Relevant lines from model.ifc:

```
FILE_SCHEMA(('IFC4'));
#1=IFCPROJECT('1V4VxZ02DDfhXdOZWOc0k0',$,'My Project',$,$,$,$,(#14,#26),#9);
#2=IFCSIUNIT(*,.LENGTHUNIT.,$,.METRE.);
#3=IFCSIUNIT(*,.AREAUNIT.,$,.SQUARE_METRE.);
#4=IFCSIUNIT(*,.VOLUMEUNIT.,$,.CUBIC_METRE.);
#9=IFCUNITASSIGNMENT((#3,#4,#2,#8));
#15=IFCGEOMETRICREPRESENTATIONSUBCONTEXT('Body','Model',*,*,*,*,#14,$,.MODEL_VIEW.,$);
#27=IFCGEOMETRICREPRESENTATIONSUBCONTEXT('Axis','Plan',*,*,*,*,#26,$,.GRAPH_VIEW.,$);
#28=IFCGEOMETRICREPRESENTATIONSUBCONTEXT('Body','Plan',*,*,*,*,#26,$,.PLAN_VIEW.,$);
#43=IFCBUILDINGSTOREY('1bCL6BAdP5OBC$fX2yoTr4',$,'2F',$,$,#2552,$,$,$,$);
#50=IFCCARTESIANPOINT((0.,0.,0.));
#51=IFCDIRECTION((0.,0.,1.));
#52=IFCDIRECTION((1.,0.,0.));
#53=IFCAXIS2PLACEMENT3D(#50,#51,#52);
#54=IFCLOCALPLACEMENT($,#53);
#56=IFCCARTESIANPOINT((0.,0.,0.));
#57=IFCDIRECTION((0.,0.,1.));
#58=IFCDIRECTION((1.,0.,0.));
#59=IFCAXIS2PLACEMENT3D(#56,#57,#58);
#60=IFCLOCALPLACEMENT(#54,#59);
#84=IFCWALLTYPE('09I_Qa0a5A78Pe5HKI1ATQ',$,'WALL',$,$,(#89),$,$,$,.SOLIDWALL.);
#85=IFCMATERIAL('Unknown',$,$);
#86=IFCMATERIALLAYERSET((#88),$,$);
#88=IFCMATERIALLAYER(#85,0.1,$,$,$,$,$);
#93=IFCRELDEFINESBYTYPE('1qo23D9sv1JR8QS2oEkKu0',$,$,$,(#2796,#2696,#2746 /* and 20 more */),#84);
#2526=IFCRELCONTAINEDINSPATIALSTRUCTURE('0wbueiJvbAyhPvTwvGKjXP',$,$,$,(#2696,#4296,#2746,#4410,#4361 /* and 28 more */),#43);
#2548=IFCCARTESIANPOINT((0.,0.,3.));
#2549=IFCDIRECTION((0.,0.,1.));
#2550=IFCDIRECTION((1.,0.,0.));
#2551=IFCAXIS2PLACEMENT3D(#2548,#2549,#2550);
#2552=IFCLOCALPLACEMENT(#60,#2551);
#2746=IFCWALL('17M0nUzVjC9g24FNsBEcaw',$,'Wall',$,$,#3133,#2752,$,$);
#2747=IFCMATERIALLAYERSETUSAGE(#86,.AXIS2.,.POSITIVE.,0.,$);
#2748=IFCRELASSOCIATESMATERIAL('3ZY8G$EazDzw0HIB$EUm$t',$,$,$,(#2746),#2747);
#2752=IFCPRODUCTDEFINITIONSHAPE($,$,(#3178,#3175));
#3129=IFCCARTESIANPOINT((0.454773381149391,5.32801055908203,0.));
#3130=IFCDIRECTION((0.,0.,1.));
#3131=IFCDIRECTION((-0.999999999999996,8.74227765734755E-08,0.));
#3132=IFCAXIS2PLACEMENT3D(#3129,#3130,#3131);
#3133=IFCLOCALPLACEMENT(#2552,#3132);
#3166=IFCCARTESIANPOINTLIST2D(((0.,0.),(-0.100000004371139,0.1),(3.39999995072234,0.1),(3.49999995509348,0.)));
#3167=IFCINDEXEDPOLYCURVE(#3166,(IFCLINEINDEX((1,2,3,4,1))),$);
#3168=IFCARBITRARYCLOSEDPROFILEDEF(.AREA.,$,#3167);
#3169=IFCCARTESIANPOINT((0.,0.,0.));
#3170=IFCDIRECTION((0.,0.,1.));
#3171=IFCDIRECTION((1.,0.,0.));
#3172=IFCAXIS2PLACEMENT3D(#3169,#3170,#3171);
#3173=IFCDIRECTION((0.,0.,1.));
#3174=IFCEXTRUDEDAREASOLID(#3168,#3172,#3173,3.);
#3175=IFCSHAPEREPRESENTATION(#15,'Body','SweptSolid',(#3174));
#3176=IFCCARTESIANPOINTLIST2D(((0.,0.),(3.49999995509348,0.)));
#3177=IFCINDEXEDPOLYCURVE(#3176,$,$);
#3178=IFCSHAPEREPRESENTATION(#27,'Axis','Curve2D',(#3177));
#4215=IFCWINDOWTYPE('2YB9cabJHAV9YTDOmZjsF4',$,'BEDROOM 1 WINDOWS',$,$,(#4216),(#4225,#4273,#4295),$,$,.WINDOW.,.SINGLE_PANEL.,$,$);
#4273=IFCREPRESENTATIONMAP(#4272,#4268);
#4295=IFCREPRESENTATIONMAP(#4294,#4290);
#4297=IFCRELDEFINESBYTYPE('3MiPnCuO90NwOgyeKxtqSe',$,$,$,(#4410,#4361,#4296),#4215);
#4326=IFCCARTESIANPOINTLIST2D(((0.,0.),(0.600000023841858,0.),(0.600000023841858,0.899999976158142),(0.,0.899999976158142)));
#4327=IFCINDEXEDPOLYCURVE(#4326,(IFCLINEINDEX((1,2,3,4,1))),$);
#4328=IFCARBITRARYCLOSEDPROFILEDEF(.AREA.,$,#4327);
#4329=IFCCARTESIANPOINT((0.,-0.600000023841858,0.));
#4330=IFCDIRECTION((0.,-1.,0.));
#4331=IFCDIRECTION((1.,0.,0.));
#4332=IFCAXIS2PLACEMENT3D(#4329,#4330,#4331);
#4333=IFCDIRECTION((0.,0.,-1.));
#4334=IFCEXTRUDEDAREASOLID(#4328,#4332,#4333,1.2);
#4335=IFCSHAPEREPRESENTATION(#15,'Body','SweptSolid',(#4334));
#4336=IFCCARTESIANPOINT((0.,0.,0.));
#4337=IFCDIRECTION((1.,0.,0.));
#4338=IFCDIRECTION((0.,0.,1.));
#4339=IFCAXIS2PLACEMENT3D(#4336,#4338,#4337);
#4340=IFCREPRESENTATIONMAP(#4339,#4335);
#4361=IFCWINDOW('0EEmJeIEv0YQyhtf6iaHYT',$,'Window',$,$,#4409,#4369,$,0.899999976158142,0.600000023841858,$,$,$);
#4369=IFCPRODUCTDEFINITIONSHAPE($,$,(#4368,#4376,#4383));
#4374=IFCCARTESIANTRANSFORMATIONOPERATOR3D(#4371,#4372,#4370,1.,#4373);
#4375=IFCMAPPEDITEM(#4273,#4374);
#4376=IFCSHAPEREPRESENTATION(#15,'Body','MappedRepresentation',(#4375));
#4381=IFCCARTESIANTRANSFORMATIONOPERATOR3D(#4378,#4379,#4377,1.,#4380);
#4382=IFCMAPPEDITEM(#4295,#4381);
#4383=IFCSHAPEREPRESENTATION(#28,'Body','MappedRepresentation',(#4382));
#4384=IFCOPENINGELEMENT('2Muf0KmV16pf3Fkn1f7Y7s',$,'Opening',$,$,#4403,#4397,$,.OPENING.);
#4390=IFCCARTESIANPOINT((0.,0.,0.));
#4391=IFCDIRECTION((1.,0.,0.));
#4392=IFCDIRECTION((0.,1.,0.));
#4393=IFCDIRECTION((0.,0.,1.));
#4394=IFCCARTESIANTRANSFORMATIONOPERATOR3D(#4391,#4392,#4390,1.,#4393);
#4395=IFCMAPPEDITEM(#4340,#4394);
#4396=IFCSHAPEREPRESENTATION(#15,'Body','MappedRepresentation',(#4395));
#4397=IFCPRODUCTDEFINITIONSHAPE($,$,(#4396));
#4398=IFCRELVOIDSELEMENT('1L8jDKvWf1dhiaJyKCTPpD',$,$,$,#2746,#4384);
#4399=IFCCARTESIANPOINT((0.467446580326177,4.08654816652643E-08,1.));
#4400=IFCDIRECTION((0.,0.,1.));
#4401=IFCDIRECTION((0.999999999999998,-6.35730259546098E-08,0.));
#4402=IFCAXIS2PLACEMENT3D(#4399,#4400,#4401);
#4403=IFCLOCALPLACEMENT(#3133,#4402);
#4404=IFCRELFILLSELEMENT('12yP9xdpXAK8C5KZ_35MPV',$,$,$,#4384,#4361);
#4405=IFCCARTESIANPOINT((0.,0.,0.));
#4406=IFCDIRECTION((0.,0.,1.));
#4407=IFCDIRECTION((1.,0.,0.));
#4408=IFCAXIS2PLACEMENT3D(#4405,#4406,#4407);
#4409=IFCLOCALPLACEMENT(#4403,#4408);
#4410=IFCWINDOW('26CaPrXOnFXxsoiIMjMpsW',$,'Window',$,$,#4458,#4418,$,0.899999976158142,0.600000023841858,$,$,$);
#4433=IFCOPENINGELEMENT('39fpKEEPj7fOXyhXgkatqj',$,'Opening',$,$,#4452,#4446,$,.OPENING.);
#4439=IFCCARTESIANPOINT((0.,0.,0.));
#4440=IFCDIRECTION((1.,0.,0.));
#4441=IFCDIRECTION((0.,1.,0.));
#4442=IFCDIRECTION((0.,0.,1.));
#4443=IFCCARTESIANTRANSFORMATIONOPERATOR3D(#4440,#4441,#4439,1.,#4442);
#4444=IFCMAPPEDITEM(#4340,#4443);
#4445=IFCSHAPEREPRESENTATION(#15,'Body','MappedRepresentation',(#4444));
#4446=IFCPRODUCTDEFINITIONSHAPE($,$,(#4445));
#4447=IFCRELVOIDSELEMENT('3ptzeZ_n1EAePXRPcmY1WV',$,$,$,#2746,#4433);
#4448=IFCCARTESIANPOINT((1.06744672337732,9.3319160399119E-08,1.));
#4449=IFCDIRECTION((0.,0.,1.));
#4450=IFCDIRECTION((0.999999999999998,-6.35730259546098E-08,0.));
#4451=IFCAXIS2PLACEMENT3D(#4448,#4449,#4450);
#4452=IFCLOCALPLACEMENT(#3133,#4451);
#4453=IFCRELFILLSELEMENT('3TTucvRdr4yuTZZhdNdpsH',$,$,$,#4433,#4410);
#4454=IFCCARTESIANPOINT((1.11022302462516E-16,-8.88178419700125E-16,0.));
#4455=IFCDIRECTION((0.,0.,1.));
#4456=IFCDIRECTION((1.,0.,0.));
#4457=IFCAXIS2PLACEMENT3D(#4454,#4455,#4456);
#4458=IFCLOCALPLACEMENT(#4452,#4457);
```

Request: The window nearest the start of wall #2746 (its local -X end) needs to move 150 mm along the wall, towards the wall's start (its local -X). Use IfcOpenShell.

```python
import ifcopenshell
import ifcopenshell.api.geometry
import ifcopenshell.util.placement

model = ifcopenshell.open("model.ifc")

window = model.by_id(4361)
opening = window.FillsVoids[0].RelatingOpeningElement
wall = opening.VoidsElements[0].RelatingBuildingElement

wall_matrix = ifcopenshell.util.placement.get_local_placement(wall.ObjectPlacement)
shift = wall_matrix[:3, 0] * -0.15
before = ifcopenshell.util.placement.get_local_placement(window.ObjectPlacement)[:3, 3].copy()

# The window is placed relative to its opening, so it follows when the opening moves.
matrix = ifcopenshell.util.placement.get_local_placement(opening.ObjectPlacement)
matrix[:3, 3] += shift
ifcopenshell.api.geometry.edit_object_placement(
    model, product=opening, matrix=matrix, is_si=False, should_transform_children=True
)

after = ifcopenshell.util.placement.get_local_placement(window.ObjectPlacement)[:3, 3]
print("window moved by", (after - before).round(3) + 0.0)

model.write("model-out.ifc")
```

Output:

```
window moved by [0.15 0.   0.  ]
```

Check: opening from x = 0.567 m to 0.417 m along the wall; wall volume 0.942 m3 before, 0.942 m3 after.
